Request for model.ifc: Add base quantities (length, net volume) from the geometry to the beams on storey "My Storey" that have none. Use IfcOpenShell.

First a look at what the model holds.

```python
import ifcopenshell
import ifcopenshell.util.element
import ifcopenshell.util.unit

model = ifcopenshell.open("model.ifc")
print(model.schema)
for unit_type in ("LENGTHUNIT", "AREAUNIT", "VOLUMEUNIT"):
    print(unit_type, ifcopenshell.util.unit.calculate_unit_scale(model, unit_type))
storey = next(s for s in model.by_type("IfcBuildingStorey") if s.Name == "My Storey")
beams = [e for e in ifcopenshell.util.element.get_decomposition(storey) if e.is_a("IfcBeam")]
for e in sorted(beams, key=lambda e: e.id()):
    print(e.id(), e.is_a(), e.Name, list(ifcopenshell.util.element.get_psets(e, qtos_only=True)), sep=" | ")
```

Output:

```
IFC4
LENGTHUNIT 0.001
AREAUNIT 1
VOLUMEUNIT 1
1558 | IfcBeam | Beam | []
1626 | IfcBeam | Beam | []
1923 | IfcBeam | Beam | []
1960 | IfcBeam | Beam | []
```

```python
import ifcopenshell
import ifcopenshell.api.pset
import ifcopenshell.geom
import ifcopenshell.util.element
import ifcopenshell.util.shape
import ifcopenshell.util.unit

model = ifcopenshell.open("model.ifc")
unit_scale = ifcopenshell.util.unit.calculate_unit_scale(model)
volume_scale = ifcopenshell.util.unit.calculate_unit_scale(model, "VOLUMEUNIT")
settings = ifcopenshell.geom.settings()

storey = next(s for s in model.by_type("IfcBuildingStorey") if s.Name == "My Storey")
beams = [e for e in ifcopenshell.util.element.get_decomposition(storey) if e.is_a("IfcBeam")]

for e in sorted(beams, key=lambda e: e.id()):
    if ifcopenshell.util.element.get_psets(e, qtos_only=True, should_inherit=False):
        continue
    # Geometry comes back in metres, in the element's own axes.
    shape = ifcopenshell.geom.create_shape(settings, e)
    values = {
        "Length": ifcopenshell.util.shape.get_max_xyz(shape.geometry) / unit_scale,
        "NetVolume": ifcopenshell.util.shape.get_volume(shape.geometry) / volume_scale,
    }
    qto = ifcopenshell.api.pset.add_qto(model, product=e, name="Qto_BeamBaseQuantities")
    ifcopenshell.api.pset.edit_qto(model, qto=qto, properties=values)
    print(e.id(), {k: round(v, 3) for k, v in values.items()})

model.write("model_rev.ifc")
```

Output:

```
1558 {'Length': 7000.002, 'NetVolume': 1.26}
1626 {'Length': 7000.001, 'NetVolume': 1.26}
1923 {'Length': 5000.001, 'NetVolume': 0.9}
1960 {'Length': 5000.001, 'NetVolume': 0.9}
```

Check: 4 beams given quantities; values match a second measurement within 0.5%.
